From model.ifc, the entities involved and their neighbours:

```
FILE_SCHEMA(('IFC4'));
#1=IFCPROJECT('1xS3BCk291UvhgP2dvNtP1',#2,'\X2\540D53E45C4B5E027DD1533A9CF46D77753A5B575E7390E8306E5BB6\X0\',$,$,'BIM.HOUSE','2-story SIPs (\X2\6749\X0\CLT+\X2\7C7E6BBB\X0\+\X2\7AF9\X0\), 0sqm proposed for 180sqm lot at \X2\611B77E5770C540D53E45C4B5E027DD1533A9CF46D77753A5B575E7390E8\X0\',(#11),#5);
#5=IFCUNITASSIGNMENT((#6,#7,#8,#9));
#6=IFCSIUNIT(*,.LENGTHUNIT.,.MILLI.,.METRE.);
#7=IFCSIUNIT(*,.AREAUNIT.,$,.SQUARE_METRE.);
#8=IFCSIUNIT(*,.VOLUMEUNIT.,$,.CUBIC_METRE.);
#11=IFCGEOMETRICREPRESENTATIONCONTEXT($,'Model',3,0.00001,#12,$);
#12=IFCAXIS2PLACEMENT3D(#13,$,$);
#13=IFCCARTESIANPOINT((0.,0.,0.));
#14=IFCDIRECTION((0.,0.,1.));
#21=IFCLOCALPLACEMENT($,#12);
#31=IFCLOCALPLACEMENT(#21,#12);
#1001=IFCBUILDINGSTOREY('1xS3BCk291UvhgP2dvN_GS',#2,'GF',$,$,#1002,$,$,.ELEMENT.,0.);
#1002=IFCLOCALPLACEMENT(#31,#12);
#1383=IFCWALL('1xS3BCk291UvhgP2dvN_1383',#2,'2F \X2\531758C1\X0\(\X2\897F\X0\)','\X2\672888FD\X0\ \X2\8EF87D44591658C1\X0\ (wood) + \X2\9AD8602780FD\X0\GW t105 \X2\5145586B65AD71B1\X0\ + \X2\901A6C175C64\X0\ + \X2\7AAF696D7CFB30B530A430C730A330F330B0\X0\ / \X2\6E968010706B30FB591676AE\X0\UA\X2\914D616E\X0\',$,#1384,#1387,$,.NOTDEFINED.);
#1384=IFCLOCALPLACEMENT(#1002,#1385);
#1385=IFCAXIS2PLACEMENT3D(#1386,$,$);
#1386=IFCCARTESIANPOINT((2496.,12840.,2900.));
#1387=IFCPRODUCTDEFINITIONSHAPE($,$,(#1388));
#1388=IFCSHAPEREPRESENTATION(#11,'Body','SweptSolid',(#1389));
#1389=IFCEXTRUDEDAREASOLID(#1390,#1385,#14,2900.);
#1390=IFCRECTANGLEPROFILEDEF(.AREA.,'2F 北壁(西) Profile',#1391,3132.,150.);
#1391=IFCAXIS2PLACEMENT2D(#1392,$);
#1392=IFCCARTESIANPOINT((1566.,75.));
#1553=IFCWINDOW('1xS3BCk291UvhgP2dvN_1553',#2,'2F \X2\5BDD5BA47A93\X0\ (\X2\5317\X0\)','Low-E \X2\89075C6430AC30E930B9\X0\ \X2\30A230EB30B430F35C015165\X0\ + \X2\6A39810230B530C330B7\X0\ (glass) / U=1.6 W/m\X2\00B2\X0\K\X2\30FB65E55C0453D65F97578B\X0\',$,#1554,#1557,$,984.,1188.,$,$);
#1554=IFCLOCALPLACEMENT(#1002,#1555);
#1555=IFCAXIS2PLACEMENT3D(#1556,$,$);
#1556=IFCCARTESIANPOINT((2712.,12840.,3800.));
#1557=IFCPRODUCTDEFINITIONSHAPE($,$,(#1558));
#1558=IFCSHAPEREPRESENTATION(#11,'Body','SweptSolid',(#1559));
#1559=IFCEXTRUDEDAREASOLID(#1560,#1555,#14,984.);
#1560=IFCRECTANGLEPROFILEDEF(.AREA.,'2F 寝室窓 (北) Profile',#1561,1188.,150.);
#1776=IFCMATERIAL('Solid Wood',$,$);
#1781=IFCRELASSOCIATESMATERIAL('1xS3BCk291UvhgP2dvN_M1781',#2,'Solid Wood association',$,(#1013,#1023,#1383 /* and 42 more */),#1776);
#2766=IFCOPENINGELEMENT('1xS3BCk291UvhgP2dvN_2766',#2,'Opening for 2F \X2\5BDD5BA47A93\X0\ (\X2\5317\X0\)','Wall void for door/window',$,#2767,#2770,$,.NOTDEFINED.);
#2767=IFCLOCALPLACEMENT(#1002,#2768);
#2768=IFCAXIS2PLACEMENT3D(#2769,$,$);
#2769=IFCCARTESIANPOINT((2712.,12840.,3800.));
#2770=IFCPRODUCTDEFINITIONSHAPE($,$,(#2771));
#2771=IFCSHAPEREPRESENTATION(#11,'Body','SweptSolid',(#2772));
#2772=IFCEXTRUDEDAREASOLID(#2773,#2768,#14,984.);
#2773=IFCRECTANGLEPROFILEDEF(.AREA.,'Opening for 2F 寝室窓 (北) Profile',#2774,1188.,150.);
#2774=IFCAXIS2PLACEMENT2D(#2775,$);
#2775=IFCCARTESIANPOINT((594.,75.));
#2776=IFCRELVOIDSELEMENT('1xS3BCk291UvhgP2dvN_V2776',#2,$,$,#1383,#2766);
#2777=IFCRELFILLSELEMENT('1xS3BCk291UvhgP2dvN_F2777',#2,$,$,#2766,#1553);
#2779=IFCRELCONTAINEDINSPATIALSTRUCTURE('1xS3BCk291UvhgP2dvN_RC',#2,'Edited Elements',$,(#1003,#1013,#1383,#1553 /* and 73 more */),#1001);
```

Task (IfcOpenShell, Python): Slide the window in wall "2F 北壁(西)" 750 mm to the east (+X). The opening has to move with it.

```python
import ifcopenshell
import ifcopenshell.api.geometry
import ifcopenshell.util.placement

model = ifcopenshell.open("model.ifc")

window = model.by_guid("1xS3BCk291UvhgP2dvN_1553")
opening = window.FillsVoids[0].RelatingOpeningElement
wall = opening.VoidsElements[0].RelatingBuildingElement

wall_matrix = ifcopenshell.util.placement.get_local_placement(wall.ObjectPlacement)
shift = wall_matrix[:3, 0] * 750.0
before = ifcopenshell.util.placement.get_local_placement(window.ObjectPlacement)[:3, 3].copy()

# The window is not placed relative to its opening, so move both.
for product in (opening, window):
    matrix = ifcopenshell.util.placement.get_local_placement(product.ObjectPlacement)
    matrix[:3, 3] += shift
    ifcopenshell.api.geometry.edit_object_placement(model, product=product, matrix=matrix, is_si=False)

after = ifcopenshell.util.placement.get_local_placement(window.ObjectPlacement)[:3, 3]
print("window moved by", (after - before).round(3) + 0.0)

model.write("model_edited.ifc")
```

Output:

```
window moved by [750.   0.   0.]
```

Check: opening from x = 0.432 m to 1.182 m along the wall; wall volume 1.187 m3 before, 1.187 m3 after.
